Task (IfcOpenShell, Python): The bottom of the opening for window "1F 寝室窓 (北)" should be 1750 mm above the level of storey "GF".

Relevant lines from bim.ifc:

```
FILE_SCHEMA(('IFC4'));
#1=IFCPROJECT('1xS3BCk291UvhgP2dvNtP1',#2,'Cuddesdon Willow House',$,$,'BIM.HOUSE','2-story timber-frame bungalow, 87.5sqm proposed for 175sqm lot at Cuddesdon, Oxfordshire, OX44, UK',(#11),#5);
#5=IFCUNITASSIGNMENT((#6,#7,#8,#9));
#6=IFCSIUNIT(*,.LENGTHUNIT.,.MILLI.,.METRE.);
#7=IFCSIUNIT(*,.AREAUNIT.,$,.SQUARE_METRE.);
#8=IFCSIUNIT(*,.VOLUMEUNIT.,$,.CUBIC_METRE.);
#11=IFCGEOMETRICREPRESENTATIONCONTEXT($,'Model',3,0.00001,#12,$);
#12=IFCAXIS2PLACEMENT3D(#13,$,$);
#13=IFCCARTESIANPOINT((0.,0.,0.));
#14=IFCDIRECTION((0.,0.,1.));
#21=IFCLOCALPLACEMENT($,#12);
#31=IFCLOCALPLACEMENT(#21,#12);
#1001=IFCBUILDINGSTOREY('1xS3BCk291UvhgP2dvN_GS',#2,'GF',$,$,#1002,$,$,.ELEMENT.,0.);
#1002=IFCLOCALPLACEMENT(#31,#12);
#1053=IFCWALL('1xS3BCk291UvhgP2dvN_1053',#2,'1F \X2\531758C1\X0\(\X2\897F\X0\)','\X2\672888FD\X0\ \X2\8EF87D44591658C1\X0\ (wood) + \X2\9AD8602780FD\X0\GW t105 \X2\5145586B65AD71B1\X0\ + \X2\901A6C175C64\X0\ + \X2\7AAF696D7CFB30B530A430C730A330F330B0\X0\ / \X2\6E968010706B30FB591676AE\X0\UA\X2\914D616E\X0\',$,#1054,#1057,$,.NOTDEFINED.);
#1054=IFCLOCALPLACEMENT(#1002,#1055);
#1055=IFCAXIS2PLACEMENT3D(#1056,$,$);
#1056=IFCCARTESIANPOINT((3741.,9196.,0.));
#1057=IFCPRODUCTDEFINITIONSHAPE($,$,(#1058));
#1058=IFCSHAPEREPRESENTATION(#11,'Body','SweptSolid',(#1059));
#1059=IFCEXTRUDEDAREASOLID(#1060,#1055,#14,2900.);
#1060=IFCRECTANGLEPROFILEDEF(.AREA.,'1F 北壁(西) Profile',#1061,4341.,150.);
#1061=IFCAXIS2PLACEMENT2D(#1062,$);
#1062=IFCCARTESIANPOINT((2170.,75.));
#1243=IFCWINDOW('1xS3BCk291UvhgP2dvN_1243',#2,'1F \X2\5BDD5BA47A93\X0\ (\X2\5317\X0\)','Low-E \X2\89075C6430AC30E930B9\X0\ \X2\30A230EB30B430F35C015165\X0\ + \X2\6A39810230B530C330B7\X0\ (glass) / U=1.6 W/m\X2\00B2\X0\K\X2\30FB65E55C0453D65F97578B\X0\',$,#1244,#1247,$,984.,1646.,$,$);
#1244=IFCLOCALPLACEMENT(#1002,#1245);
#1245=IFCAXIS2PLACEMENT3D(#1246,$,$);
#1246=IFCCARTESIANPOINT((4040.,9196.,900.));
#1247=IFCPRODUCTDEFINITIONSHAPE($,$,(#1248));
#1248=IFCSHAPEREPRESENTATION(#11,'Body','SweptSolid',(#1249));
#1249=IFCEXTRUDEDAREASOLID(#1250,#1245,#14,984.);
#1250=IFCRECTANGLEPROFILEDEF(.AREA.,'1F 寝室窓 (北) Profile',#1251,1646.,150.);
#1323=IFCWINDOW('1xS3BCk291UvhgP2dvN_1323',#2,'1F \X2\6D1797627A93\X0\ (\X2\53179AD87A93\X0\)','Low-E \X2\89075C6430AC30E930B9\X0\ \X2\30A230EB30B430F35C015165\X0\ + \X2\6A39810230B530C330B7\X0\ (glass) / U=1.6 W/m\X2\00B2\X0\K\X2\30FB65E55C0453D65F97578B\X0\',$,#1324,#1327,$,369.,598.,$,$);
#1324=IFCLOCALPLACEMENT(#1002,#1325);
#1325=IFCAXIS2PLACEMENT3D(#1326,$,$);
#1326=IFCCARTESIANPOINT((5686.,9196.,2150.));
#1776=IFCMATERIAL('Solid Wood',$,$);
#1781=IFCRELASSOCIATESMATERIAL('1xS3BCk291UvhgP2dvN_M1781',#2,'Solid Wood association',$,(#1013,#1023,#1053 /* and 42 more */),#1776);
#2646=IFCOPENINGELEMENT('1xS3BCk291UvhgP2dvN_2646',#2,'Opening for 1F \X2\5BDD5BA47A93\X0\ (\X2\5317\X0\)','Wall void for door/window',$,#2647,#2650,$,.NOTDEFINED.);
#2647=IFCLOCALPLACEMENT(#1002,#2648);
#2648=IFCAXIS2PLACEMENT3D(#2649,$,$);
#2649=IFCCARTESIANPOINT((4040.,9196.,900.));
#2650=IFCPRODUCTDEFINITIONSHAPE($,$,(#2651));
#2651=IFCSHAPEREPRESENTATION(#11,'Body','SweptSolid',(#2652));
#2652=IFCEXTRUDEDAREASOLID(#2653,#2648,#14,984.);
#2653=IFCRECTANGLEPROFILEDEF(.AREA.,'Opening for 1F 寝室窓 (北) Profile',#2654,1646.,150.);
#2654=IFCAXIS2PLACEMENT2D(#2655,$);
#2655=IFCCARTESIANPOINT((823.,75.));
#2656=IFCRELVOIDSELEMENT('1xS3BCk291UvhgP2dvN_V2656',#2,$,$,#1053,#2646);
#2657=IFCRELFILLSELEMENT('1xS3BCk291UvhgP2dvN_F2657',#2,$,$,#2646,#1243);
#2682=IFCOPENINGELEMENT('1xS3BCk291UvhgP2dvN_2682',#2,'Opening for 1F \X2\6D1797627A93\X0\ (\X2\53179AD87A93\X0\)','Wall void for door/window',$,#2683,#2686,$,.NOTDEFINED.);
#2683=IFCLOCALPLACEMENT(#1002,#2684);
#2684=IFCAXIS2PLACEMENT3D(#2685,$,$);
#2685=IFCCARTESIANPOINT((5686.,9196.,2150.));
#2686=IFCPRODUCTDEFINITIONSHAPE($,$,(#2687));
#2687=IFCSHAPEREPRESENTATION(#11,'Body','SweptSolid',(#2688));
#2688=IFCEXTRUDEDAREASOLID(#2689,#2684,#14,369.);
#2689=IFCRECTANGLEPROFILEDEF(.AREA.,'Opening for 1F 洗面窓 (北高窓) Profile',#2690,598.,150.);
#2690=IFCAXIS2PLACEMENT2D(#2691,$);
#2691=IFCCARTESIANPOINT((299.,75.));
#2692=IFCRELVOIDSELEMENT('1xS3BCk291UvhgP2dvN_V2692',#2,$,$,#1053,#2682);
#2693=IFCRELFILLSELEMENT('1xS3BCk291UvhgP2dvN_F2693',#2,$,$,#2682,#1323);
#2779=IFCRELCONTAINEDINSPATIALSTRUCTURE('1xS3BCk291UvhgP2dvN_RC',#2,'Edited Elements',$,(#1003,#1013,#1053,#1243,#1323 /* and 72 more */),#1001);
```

```python
import numpy as np
import ifcopenshell
import ifcopenshell.api.geometry
import ifcopenshell.geom
import ifcopenshell.util.element
import ifcopenshell.util.placement
import ifcopenshell.util.shape
import ifcopenshell.util.unit

model = ifcopenshell.open("bim.ifc")
unit_scale = ifcopenshell.util.unit.calculate_unit_scale(model)

window = model.by_guid("1xS3BCk291UvhgP2dvN_1243")
opening = window.FillsVoids[0].RelatingOpeningElement
storey = ifcopenshell.util.element.get_container(window, ifc_class="IfcBuildingStorey")
level = ifcopenshell.util.placement.get_local_placement(storey.ObjectPlacement)[2, 3]

# The opening's origin need not be at the sill, so measure its lowest point.
shape = ifcopenshell.geom.create_shape(ifcopenshell.geom.settings(), opening)
bottom = ifcopenshell.util.shape.get_shape_bottom_elevation(shape, shape.geometry) / unit_scale
dz = level + 1.75 / unit_scale - bottom

shift = np.array([0.0, 0.0, dz])
# The window is not placed relative to its opening, so move both.
for product in (opening, window):
    matrix = ifcopenshell.util.placement.get_local_placement(product.ObjectPlacement)
    matrix[:3, 3] += shift
    ifcopenshell.api.geometry.edit_object_placement(model, product=product, matrix=matrix, is_si=False)

print(f"moved by {dz * unit_scale:+.3f} m")

model.write("bim_rev.ifc")
```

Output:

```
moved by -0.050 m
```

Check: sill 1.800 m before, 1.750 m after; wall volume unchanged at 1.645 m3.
